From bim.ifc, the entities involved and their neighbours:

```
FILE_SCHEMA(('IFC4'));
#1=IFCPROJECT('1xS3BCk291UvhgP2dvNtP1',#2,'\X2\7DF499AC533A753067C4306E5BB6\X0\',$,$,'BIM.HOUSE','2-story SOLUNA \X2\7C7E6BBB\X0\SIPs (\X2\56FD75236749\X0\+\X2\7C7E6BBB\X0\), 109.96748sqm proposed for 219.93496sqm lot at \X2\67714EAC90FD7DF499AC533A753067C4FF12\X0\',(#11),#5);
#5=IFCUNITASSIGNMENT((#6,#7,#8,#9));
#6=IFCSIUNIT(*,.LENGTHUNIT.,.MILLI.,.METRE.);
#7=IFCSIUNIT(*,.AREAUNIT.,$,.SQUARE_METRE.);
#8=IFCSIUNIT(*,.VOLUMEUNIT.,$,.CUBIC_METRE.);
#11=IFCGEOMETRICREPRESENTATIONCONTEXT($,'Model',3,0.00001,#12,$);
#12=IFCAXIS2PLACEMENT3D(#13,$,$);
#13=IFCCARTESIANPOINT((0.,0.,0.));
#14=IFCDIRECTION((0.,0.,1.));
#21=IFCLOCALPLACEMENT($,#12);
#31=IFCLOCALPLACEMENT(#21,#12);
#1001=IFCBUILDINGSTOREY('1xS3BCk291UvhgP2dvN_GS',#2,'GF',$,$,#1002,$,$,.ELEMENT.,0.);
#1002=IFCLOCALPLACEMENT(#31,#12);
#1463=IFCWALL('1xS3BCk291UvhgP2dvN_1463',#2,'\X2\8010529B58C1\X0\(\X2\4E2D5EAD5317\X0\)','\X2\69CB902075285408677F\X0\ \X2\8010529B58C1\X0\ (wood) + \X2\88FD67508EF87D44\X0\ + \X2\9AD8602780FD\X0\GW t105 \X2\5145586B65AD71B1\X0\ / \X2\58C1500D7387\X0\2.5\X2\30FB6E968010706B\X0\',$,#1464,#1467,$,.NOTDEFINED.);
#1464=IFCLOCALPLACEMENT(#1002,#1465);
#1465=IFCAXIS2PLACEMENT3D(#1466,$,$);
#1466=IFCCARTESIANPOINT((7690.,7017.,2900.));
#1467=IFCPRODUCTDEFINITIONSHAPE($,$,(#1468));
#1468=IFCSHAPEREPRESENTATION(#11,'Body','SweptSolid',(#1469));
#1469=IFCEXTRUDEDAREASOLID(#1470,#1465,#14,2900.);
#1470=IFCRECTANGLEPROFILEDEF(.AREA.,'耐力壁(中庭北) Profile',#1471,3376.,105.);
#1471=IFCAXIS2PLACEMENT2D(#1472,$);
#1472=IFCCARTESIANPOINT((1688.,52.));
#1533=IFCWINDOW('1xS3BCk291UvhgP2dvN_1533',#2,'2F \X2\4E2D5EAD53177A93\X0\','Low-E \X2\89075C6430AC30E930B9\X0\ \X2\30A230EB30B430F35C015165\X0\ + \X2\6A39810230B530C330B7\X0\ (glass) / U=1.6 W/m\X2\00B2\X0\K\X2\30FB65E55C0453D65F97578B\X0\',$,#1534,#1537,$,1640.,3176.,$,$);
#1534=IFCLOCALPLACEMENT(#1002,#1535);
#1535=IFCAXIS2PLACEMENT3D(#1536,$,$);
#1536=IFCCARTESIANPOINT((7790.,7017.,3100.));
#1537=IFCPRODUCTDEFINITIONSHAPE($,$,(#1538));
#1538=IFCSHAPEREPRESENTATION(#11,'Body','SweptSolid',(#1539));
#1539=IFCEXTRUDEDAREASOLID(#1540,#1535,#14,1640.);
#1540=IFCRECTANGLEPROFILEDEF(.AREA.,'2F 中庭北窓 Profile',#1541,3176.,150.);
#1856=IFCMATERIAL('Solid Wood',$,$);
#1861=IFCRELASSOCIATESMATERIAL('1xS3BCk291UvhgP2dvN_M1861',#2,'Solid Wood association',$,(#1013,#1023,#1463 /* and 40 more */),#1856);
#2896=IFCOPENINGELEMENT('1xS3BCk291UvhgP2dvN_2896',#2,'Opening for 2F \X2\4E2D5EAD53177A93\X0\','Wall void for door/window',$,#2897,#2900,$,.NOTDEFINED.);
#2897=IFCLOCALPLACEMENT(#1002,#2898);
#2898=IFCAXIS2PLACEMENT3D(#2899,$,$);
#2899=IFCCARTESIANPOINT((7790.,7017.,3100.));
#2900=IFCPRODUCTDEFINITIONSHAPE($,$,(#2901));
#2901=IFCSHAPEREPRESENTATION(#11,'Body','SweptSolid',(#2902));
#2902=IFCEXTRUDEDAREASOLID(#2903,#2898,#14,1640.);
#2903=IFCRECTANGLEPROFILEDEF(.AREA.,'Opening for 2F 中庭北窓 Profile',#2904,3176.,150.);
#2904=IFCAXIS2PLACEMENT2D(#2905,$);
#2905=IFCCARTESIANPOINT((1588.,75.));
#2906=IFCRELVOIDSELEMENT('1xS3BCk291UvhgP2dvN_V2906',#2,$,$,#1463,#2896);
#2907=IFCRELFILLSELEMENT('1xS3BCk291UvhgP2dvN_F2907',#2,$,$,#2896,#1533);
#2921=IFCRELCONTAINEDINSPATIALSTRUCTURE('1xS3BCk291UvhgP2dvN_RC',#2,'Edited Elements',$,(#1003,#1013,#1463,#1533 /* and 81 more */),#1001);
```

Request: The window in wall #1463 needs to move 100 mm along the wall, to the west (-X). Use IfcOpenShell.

```python
import ifcopenshell
import ifcopenshell.api.geometry
import ifcopenshell.util.placement

model = ifcopenshell.open("bim.ifc")

window = model.by_id(1533)
opening = window.FillsVoids[0].RelatingOpeningElement
wall = opening.VoidsElements[0].RelatingBuildingElement

wall_matrix = ifcopenshell.util.placement.get_local_placement(wall.ObjectPlacement)
shift = wall_matrix[:3, 0] * -100.0
before = ifcopenshell.util.placement.get_local_placement(window.ObjectPlacement)[:3, 3].copy()

# The window is not placed relative to its opening, so move both.
for product in (opening, window):
    matrix = ifcopenshell.util.placement.get_local_placement(product.ObjectPlacement)
    matrix[:3, 3] += shift
    ifcopenshell.api.geometry.edit_object_placement(model, product=product, matrix=matrix, is_si=False)

after = ifcopenshell.util.placement.get_local_placement(window.ObjectPlacement)[:3, 3]
print("window moved by", (after - before).round(3) + 0.0)

model.write("bim_edited.ifc")
```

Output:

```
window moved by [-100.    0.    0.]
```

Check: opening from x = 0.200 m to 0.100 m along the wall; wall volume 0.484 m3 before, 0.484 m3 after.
